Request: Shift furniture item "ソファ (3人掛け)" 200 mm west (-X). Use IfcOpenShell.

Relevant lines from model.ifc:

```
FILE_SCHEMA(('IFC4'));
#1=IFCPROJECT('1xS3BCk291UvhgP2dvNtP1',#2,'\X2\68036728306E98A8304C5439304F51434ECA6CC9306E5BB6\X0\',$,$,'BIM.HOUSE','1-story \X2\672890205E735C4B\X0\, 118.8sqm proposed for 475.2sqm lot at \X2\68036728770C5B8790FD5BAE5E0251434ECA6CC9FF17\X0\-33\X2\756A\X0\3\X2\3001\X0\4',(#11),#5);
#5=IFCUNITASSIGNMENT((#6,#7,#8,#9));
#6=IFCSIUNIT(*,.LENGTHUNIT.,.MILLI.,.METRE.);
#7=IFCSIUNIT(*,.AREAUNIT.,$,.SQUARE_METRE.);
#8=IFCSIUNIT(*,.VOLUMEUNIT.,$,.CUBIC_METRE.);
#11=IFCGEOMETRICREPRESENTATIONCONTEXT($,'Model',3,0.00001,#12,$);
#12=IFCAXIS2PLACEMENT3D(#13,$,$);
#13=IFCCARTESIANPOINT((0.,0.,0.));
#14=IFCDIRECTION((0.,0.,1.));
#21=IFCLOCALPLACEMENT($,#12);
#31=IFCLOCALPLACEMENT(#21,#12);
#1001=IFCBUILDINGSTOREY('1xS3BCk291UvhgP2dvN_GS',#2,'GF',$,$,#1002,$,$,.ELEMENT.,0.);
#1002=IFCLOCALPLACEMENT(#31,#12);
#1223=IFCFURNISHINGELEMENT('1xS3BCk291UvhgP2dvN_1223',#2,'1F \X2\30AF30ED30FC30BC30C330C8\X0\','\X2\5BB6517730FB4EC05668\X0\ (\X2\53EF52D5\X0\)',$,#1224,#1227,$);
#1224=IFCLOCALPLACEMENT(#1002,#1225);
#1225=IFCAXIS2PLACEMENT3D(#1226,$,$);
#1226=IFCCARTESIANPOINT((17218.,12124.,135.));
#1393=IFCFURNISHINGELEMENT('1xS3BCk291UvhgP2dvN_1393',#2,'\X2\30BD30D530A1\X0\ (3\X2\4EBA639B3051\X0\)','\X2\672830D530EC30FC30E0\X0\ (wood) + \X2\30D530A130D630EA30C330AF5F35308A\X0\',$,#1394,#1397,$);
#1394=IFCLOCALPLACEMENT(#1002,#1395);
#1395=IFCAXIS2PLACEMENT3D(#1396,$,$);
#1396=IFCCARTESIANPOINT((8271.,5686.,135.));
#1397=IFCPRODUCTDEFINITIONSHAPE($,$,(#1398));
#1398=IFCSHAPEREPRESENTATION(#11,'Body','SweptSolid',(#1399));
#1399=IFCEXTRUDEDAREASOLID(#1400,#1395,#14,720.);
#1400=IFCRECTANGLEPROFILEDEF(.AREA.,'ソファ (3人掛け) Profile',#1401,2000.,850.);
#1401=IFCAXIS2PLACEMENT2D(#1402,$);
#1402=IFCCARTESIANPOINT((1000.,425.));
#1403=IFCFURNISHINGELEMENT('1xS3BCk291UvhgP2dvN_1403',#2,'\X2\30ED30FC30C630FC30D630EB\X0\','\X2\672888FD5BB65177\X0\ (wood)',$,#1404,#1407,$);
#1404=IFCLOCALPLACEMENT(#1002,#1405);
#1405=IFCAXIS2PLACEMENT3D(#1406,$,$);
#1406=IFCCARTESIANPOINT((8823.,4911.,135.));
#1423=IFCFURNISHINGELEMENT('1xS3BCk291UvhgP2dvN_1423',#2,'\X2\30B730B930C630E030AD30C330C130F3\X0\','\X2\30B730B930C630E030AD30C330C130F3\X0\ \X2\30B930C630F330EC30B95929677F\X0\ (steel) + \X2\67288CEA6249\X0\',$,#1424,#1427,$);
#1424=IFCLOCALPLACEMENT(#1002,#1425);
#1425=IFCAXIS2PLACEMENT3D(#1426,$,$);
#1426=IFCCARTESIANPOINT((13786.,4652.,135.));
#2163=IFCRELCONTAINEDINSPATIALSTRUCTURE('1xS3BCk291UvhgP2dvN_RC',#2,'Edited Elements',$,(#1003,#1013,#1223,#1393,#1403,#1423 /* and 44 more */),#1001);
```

```python
import ifcopenshell
import ifcopenshell.api.geometry
import ifcopenshell.util.placement

model = ifcopenshell.open("model.ifc")

item = model.by_guid("1xS3BCk291UvhgP2dvN_1393")
matrix = ifcopenshell.util.placement.get_local_placement(item.ObjectPlacement)
matrix[0, 3] -= 200.0
ifcopenshell.api.geometry.edit_object_placement(model, product=item, matrix=matrix, is_si=False)

print(ifcopenshell.util.placement.get_local_placement(item.ObjectPlacement).round(3) + 0.0)

model.write("model_v2.ifc")
```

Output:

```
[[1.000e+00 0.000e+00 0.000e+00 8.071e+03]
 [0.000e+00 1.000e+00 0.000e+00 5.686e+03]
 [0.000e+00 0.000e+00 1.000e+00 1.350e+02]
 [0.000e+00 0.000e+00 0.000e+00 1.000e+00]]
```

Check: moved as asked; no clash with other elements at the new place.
